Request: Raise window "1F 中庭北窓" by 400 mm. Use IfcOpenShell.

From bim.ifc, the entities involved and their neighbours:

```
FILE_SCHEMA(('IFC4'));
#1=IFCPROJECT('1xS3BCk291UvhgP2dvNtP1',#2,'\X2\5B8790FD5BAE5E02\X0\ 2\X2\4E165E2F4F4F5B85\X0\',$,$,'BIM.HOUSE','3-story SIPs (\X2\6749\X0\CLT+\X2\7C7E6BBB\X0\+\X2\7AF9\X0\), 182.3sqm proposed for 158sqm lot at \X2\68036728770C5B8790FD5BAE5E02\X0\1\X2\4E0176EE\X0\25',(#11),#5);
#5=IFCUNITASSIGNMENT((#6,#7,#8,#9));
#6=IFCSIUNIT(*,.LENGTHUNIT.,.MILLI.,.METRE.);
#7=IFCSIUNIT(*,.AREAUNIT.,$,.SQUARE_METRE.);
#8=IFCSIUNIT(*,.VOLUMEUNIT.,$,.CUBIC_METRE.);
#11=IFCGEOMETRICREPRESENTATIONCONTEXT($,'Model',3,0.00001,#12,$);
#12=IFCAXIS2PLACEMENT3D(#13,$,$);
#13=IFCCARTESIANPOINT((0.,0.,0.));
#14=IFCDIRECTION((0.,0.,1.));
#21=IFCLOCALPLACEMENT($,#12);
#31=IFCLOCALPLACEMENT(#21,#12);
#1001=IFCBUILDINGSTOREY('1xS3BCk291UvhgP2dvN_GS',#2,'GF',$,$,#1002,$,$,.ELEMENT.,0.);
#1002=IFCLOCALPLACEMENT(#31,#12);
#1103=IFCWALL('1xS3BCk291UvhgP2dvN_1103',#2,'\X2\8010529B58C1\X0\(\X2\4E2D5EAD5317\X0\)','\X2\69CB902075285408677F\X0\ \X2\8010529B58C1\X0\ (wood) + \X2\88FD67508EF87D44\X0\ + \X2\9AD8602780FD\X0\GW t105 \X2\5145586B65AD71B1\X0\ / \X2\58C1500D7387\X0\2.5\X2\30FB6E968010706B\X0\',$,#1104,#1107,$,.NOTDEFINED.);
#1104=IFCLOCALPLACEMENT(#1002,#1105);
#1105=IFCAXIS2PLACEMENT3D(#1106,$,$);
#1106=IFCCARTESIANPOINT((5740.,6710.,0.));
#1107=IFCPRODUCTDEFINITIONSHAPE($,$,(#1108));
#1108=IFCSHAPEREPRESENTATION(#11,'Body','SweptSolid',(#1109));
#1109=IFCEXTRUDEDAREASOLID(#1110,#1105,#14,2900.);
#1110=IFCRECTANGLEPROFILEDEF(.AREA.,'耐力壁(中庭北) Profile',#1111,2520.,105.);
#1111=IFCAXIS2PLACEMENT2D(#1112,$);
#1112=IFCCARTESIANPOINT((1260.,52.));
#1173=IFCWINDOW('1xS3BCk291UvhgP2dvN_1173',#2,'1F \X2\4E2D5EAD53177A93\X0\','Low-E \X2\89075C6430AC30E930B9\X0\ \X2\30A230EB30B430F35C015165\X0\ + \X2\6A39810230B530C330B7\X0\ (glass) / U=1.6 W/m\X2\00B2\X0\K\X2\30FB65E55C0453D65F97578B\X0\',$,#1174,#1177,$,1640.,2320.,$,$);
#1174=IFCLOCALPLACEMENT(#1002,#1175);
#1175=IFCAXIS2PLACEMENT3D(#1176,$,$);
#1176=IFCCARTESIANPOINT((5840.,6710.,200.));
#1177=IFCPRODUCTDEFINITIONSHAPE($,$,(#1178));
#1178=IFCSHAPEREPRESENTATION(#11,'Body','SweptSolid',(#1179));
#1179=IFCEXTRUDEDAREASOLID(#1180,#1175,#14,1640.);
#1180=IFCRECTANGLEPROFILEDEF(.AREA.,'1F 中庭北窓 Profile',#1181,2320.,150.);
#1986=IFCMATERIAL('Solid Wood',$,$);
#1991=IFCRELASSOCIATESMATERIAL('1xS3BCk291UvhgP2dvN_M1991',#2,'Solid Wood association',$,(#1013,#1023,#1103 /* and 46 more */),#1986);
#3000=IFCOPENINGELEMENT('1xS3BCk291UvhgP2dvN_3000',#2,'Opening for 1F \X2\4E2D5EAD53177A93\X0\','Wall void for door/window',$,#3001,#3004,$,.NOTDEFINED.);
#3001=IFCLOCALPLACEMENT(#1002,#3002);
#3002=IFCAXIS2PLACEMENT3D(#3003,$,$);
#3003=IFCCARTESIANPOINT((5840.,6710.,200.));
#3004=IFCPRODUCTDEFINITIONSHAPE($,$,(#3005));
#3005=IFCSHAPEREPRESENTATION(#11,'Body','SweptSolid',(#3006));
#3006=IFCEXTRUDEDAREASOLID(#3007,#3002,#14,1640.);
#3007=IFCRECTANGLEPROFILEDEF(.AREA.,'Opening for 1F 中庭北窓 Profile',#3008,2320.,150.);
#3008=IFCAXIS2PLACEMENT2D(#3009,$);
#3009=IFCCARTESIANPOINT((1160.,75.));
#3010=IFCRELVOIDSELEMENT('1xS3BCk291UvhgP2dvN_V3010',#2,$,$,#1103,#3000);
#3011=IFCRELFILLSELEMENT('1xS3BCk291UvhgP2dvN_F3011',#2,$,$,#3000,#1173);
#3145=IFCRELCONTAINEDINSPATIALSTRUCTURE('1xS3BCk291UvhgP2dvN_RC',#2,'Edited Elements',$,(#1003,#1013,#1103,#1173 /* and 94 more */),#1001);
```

```python
import numpy as np
import ifcopenshell
import ifcopenshell.api.geometry
import ifcopenshell.util.placement
import ifcopenshell.util.unit

model = ifcopenshell.open("bim.ifc")
unit_scale = ifcopenshell.util.unit.calculate_unit_scale(model)

window = model.by_guid("1xS3BCk291UvhgP2dvN_1173")
opening = window.FillsVoids[0].RelatingOpeningElement
dz = 0.4 / unit_scale

shift = np.array([0.0, 0.0, dz])
# The window is not placed relative to its opening, so move both.
for product in (opening, window):
    matrix = ifcopenshell.util.placement.get_local_placement(product.ObjectPlacement)
    matrix[:3, 3] += shift
    ifcopenshell.api.geometry.edit_object_placement(model, product=product, matrix=matrix, is_si=False)

print(f"moved by {dz * unit_scale:+.3f} m")

model.write("bim_rev.ifc")
```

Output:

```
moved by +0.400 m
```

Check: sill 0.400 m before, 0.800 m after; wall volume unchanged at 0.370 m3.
